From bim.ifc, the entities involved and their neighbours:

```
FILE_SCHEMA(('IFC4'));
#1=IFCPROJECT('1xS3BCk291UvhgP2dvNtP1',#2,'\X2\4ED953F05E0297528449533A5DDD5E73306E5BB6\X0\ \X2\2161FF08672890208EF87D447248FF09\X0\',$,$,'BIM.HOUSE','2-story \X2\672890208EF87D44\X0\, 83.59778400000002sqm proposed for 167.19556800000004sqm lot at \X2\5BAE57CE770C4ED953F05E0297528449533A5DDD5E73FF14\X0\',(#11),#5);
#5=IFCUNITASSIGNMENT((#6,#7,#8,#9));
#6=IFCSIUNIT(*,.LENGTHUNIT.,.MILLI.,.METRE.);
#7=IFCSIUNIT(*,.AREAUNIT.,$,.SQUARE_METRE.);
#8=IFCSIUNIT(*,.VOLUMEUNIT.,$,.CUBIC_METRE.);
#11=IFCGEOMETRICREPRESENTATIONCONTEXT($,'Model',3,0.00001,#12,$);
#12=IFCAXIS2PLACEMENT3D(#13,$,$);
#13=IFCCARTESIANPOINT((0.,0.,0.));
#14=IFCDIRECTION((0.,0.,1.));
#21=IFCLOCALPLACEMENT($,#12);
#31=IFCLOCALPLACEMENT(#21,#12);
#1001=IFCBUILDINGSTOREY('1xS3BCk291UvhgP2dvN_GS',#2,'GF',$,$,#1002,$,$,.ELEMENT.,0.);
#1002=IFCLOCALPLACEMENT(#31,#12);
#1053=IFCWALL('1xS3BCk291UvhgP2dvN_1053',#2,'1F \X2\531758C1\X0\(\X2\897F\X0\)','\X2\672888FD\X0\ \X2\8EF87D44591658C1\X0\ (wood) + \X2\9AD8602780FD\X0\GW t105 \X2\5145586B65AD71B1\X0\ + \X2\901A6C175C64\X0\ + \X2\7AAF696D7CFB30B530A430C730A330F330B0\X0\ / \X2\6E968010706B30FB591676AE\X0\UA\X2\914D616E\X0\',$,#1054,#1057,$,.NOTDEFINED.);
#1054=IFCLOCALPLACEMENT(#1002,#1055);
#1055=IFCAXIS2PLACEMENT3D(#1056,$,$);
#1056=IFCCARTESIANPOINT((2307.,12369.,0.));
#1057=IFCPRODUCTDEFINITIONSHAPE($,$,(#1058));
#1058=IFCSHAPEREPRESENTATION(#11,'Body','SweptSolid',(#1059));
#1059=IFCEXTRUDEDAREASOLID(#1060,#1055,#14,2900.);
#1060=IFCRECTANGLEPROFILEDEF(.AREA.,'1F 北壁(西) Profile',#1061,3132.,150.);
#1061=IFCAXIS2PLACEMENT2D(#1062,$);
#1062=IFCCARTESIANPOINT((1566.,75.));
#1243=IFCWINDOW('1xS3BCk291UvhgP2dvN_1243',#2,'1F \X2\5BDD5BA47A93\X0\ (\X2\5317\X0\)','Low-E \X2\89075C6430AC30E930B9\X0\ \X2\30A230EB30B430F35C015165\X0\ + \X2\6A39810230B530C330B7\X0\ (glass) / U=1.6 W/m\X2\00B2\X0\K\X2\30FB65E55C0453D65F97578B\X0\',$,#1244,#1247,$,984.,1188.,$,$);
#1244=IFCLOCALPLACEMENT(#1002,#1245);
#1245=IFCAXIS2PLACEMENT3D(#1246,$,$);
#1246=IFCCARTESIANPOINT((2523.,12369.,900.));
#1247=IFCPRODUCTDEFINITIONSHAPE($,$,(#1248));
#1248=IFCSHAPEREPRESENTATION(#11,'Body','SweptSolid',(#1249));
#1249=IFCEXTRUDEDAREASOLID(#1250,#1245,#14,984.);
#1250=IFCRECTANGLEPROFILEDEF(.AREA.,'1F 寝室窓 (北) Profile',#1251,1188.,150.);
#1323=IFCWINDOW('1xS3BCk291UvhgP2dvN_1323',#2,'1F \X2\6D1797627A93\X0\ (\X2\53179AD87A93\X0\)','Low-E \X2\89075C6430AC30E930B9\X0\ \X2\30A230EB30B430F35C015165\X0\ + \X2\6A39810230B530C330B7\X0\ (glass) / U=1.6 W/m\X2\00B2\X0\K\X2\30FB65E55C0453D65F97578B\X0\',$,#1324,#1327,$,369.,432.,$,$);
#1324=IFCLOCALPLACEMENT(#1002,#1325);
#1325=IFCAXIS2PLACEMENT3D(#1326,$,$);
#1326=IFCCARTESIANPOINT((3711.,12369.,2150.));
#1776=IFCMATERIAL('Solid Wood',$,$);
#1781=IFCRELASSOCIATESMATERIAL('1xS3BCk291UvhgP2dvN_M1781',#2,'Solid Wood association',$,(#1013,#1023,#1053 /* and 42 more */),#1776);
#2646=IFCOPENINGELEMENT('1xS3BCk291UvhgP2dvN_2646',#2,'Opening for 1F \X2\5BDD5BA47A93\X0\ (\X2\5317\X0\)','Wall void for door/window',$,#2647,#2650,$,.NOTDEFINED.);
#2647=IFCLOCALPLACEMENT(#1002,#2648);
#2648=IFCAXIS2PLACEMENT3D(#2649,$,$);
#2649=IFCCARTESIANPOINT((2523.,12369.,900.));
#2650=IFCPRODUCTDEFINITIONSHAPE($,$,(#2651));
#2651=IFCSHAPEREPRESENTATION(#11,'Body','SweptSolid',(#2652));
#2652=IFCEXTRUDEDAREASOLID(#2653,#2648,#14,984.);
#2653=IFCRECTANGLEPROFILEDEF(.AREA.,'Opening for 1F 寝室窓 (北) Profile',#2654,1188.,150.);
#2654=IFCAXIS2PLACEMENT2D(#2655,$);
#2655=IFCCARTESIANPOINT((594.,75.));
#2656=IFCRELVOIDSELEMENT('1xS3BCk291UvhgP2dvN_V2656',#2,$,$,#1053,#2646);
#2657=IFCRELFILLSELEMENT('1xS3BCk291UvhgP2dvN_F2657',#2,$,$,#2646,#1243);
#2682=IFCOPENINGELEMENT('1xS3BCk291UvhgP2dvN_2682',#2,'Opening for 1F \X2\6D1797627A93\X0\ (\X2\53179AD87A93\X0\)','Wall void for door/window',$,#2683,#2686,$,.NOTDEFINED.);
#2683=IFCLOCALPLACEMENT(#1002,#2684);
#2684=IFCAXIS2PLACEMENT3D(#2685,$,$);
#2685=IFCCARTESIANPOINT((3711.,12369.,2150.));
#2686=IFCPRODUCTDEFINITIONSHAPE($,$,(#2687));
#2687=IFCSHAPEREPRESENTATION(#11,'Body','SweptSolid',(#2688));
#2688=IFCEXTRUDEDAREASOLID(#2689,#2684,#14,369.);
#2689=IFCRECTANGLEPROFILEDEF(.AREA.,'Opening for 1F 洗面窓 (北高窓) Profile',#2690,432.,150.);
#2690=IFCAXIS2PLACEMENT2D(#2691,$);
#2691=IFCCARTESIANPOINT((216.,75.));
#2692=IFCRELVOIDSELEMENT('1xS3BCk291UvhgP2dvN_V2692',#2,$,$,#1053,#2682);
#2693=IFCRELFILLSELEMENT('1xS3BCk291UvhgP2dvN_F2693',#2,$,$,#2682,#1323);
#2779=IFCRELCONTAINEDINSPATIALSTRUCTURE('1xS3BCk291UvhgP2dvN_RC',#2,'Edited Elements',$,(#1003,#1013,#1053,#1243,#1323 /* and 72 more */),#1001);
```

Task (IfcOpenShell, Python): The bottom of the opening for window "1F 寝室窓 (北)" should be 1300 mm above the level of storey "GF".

```python
import numpy as np
import ifcopenshell
import ifcopenshell.api.geometry
import ifcopenshell.geom
import ifcopenshell.util.element
import ifcopenshell.util.placement
import ifcopenshell.util.shape
import ifcopenshell.util.unit

model = ifcopenshell.open("bim.ifc")
unit_scale = ifcopenshell.util.unit.calculate_unit_scale(model)

window = model.by_id(1243)
opening = window.FillsVoids[0].RelatingOpeningElement
storey = ifcopenshell.util.element.get_container(window, ifc_class="IfcBuildingStorey")
level = ifcopenshell.util.placement.get_local_placement(storey.ObjectPlacement)[2, 3]

# The opening's origin need not be at the sill, so measure its lowest point.
shape = ifcopenshell.geom.create_shape(ifcopenshell.geom.settings(), opening)
bottom = ifcopenshell.util.shape.get_shape_bottom_elevation(shape, shape.geometry) / unit_scale
dz = level + 1.3 / unit_scale - bottom

shift = np.array([0.0, 0.0, dz])
# The window is not placed relative to its opening, so move both.
for product in (opening, window):
    matrix = ifcopenshell.util.placement.get_local_placement(product.ObjectPlacement)
    matrix[:3, 3] += shift
    ifcopenshell.api.geometry.edit_object_placement(model, product=product, matrix=matrix, is_si=False)

print(f"moved by {dz * unit_scale:+.3f} m")

model.write("bim_edited.ifc")
```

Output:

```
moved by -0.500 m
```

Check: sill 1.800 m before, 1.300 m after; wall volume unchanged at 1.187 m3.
